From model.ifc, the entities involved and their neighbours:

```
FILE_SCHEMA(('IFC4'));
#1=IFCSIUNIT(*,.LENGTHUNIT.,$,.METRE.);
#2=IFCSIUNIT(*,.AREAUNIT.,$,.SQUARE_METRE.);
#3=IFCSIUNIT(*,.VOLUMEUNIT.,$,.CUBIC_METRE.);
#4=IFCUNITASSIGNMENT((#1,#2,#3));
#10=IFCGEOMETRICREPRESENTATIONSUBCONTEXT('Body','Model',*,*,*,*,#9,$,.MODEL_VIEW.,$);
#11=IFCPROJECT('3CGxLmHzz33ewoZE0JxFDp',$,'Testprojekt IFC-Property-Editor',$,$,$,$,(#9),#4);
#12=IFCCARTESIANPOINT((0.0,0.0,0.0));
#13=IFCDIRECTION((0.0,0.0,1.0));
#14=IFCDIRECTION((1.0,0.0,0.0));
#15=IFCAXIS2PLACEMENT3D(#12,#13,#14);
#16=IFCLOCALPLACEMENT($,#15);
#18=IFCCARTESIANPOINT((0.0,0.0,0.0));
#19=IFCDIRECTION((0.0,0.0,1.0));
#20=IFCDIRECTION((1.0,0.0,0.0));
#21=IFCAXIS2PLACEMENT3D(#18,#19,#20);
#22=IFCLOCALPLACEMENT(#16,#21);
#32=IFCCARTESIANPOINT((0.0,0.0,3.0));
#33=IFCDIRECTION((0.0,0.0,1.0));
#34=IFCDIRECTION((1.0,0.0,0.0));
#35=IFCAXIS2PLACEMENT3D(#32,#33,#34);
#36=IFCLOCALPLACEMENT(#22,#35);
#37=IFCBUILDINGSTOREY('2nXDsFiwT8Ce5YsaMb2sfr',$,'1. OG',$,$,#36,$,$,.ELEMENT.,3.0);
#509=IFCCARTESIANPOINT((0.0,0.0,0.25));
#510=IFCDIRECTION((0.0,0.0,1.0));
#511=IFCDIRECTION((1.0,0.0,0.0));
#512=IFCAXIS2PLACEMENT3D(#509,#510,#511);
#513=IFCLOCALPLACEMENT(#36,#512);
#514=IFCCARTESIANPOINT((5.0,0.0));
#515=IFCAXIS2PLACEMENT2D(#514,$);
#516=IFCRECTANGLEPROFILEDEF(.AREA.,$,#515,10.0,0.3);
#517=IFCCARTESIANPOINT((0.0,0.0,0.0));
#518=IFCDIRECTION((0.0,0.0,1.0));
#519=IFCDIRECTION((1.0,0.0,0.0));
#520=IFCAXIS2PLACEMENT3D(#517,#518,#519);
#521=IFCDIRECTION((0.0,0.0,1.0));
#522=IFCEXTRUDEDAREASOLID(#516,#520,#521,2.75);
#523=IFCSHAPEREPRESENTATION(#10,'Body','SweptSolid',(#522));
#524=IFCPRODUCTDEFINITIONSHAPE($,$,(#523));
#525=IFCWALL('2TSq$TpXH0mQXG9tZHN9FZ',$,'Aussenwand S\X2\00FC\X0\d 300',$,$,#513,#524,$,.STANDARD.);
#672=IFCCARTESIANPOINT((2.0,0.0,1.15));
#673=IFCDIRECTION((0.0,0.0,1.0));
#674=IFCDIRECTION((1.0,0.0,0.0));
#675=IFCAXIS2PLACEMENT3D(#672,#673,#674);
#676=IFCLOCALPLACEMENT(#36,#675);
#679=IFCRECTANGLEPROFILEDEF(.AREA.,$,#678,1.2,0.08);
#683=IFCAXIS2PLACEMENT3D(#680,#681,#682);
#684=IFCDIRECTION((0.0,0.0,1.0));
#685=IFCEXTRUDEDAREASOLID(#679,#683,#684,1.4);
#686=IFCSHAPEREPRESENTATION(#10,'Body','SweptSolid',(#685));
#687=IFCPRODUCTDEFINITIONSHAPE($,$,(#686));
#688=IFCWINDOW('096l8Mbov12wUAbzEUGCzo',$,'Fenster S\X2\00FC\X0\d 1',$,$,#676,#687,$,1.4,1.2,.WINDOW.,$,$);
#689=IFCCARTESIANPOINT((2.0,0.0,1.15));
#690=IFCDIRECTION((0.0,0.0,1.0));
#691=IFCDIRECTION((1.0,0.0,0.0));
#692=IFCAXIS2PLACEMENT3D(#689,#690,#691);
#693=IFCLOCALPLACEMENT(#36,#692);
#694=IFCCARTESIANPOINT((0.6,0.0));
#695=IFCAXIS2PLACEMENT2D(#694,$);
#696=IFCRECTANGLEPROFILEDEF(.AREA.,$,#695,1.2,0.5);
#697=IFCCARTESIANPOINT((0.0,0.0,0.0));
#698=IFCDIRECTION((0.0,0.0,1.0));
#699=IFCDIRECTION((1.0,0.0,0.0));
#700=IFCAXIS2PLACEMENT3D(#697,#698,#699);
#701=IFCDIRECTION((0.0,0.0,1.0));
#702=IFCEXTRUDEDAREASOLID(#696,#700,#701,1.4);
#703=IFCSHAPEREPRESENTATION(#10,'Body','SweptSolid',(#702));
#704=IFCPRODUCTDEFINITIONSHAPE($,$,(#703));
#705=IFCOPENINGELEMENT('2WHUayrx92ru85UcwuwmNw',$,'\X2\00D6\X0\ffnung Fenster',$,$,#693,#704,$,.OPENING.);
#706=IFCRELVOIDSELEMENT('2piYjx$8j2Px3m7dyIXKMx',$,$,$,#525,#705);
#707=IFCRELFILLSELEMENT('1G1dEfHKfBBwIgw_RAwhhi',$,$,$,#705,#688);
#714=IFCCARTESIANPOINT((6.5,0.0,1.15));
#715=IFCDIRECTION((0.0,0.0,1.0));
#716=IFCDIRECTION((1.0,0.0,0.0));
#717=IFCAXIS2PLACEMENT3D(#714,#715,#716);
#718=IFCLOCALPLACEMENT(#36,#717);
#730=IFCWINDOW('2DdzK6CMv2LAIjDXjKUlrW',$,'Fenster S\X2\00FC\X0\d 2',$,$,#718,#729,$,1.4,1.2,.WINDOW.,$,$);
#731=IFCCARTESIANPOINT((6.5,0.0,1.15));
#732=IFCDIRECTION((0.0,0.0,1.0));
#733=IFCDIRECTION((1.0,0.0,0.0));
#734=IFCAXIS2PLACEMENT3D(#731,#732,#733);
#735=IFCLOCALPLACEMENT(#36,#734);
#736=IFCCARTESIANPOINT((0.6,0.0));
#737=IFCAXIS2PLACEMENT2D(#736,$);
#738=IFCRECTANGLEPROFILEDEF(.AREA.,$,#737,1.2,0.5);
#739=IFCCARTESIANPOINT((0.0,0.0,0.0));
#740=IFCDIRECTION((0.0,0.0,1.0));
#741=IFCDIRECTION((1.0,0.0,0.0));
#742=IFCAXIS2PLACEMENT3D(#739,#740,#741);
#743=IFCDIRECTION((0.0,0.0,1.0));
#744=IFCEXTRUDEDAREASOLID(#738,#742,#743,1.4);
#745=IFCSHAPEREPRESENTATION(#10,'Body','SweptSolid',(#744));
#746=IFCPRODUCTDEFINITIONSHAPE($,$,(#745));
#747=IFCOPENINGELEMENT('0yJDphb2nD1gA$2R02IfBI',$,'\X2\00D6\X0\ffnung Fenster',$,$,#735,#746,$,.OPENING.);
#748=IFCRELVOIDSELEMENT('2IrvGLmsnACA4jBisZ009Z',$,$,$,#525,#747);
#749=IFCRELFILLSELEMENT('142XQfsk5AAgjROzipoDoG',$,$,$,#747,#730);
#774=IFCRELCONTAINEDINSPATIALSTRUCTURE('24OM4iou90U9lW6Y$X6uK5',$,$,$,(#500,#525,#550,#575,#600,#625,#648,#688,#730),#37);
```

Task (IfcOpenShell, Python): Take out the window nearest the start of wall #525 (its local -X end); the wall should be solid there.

```python
import ifcopenshell
import ifcopenshell.api.feature
import ifcopenshell.api.root
import ifcopenshell.geom
import ifcopenshell.util.shape

model = ifcopenshell.open("model.ifc")
settings = ifcopenshell.geom.settings()


def volume(element):
    """Net volume in cubic metres, openings subtracted."""
    shape = ifcopenshell.geom.create_shape(settings, element)
    return ifcopenshell.util.shape.get_volume(shape.geometry)


window = model.by_guid("096l8Mbov12wUAbzEUGCzo")
opening = window.FillsVoids[0].RelatingOpeningElement
wall = opening.VoidsElements[0].RelatingBuildingElement
before = volume(wall)

ifcopenshell.api.root.remove_product(model, product=window)
ifcopenshell.api.feature.remove_feature(model, feature=opening)

after = volume(wall)

print(f"wall volume {before:.3f} -> {after:.3f} m3")

model.write("model-out.ifc")
```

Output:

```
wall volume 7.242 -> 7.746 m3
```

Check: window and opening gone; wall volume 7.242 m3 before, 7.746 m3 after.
